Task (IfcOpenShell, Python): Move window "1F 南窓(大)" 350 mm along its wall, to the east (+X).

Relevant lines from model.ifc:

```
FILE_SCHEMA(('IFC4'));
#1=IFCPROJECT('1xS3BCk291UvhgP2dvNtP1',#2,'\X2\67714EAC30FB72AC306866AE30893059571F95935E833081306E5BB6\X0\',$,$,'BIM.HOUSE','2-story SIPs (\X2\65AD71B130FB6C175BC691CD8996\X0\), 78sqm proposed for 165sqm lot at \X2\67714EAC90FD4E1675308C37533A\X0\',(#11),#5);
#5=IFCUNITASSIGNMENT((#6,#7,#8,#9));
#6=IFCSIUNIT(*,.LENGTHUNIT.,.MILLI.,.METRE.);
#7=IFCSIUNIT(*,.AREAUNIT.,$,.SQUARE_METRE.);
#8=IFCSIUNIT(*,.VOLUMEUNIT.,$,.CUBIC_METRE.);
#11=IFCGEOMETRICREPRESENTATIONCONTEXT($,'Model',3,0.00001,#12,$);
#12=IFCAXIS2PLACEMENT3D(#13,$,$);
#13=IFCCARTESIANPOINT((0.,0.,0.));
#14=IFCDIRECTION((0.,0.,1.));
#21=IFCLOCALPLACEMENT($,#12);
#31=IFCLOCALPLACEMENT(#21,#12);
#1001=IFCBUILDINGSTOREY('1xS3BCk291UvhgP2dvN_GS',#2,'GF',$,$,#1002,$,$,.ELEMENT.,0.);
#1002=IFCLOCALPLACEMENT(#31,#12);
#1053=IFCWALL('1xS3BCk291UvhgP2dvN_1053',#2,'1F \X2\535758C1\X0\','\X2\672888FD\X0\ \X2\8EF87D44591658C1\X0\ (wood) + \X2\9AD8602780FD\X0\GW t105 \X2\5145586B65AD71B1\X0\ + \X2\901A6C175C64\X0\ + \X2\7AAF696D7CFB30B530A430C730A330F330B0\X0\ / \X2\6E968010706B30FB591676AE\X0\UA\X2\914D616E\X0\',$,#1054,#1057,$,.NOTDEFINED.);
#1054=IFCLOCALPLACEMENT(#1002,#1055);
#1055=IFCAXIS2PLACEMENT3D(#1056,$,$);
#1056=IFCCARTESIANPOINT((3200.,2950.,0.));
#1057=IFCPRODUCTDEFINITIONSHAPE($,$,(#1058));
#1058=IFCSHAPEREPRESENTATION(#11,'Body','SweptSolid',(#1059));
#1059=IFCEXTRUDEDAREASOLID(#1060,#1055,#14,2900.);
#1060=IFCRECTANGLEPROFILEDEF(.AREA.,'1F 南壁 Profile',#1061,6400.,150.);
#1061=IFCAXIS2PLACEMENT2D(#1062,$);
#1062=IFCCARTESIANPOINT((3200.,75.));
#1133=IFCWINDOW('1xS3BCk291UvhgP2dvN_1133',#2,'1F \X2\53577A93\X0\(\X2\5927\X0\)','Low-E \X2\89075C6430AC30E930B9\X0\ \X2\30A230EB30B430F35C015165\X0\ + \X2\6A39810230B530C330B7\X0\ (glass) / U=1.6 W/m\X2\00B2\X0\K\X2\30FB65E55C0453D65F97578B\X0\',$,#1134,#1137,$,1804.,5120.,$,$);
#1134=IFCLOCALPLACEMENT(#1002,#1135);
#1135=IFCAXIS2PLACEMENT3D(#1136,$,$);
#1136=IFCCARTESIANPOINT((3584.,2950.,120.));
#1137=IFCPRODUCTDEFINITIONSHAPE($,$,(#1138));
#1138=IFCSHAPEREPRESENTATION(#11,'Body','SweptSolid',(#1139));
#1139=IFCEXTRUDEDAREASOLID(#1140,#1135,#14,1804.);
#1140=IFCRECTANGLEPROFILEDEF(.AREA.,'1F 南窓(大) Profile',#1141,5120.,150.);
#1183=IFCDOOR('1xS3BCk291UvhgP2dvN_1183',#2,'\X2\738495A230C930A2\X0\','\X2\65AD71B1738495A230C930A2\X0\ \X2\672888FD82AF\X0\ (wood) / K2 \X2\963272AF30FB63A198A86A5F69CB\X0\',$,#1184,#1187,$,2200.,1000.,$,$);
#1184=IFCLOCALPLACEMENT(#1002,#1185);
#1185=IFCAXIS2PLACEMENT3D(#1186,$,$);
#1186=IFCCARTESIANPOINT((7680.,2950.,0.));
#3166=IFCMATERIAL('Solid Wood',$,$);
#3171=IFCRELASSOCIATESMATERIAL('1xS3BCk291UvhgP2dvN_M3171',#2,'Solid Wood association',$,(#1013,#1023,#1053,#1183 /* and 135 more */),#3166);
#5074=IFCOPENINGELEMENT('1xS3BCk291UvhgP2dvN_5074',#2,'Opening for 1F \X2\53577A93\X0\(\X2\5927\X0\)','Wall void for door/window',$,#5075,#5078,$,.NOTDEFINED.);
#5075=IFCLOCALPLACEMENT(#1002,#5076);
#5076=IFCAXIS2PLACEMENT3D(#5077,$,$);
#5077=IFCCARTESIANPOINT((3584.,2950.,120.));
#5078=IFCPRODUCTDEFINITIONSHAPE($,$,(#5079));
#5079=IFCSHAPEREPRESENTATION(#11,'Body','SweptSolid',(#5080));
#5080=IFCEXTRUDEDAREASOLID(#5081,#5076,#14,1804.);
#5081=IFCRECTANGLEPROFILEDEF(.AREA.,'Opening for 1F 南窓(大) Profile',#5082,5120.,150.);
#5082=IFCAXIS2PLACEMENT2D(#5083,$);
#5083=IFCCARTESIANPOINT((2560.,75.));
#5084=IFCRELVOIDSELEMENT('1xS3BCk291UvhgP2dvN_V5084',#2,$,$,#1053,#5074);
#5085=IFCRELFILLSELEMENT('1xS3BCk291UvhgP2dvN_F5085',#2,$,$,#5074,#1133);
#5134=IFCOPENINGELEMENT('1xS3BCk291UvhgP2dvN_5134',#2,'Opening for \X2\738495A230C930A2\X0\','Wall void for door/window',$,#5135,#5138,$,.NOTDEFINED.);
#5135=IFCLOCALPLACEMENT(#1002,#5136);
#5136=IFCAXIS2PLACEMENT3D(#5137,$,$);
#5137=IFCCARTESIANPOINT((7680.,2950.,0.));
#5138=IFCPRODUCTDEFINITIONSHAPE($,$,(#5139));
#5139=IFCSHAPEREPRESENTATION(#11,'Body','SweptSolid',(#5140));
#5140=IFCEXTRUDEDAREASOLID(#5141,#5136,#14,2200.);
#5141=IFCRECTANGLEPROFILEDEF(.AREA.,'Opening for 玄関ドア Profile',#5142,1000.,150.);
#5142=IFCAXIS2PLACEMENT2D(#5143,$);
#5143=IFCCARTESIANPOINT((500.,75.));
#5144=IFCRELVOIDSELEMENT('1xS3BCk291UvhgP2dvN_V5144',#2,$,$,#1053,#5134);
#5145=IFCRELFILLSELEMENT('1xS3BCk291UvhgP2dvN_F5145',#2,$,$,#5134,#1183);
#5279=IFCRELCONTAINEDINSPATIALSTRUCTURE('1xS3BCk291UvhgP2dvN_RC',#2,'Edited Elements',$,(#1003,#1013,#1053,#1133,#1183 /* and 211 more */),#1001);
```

```python
import ifcopenshell
import ifcopenshell.api.geometry
import ifcopenshell.util.placement
import ifcopenshell.util.unit

model = ifcopenshell.open("model.ifc")
unit_scale = ifcopenshell.util.unit.calculate_unit_scale(model)

window = model.by_guid("1xS3BCk291UvhgP2dvN_1133")
opening = window.FillsVoids[0].RelatingOpeningElement
wall = opening.VoidsElements[0].RelatingBuildingElement

wall_matrix = ifcopenshell.util.placement.get_local_placement(wall.ObjectPlacement)
shift = wall_matrix[:3, 0] * 0.35 / unit_scale
before = ifcopenshell.util.placement.get_local_placement(window.ObjectPlacement)[:3, 3].copy()

# The window is not placed relative to its opening, so move both.
for product in (opening, window):
    matrix = ifcopenshell.util.placement.get_local_placement(product.ObjectPlacement)
    matrix[:3, 3] += shift
    ifcopenshell.api.geometry.edit_object_placement(model, product=product, matrix=matrix, is_si=False)

after = ifcopenshell.util.placement.get_local_placement(window.ObjectPlacement)[:3, 3]
print("window moved by", (after - before).round(3) + 0.0)

model.write("model-out.ifc")
```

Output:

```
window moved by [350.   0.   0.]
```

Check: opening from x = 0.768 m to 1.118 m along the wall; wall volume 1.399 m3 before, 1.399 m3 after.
